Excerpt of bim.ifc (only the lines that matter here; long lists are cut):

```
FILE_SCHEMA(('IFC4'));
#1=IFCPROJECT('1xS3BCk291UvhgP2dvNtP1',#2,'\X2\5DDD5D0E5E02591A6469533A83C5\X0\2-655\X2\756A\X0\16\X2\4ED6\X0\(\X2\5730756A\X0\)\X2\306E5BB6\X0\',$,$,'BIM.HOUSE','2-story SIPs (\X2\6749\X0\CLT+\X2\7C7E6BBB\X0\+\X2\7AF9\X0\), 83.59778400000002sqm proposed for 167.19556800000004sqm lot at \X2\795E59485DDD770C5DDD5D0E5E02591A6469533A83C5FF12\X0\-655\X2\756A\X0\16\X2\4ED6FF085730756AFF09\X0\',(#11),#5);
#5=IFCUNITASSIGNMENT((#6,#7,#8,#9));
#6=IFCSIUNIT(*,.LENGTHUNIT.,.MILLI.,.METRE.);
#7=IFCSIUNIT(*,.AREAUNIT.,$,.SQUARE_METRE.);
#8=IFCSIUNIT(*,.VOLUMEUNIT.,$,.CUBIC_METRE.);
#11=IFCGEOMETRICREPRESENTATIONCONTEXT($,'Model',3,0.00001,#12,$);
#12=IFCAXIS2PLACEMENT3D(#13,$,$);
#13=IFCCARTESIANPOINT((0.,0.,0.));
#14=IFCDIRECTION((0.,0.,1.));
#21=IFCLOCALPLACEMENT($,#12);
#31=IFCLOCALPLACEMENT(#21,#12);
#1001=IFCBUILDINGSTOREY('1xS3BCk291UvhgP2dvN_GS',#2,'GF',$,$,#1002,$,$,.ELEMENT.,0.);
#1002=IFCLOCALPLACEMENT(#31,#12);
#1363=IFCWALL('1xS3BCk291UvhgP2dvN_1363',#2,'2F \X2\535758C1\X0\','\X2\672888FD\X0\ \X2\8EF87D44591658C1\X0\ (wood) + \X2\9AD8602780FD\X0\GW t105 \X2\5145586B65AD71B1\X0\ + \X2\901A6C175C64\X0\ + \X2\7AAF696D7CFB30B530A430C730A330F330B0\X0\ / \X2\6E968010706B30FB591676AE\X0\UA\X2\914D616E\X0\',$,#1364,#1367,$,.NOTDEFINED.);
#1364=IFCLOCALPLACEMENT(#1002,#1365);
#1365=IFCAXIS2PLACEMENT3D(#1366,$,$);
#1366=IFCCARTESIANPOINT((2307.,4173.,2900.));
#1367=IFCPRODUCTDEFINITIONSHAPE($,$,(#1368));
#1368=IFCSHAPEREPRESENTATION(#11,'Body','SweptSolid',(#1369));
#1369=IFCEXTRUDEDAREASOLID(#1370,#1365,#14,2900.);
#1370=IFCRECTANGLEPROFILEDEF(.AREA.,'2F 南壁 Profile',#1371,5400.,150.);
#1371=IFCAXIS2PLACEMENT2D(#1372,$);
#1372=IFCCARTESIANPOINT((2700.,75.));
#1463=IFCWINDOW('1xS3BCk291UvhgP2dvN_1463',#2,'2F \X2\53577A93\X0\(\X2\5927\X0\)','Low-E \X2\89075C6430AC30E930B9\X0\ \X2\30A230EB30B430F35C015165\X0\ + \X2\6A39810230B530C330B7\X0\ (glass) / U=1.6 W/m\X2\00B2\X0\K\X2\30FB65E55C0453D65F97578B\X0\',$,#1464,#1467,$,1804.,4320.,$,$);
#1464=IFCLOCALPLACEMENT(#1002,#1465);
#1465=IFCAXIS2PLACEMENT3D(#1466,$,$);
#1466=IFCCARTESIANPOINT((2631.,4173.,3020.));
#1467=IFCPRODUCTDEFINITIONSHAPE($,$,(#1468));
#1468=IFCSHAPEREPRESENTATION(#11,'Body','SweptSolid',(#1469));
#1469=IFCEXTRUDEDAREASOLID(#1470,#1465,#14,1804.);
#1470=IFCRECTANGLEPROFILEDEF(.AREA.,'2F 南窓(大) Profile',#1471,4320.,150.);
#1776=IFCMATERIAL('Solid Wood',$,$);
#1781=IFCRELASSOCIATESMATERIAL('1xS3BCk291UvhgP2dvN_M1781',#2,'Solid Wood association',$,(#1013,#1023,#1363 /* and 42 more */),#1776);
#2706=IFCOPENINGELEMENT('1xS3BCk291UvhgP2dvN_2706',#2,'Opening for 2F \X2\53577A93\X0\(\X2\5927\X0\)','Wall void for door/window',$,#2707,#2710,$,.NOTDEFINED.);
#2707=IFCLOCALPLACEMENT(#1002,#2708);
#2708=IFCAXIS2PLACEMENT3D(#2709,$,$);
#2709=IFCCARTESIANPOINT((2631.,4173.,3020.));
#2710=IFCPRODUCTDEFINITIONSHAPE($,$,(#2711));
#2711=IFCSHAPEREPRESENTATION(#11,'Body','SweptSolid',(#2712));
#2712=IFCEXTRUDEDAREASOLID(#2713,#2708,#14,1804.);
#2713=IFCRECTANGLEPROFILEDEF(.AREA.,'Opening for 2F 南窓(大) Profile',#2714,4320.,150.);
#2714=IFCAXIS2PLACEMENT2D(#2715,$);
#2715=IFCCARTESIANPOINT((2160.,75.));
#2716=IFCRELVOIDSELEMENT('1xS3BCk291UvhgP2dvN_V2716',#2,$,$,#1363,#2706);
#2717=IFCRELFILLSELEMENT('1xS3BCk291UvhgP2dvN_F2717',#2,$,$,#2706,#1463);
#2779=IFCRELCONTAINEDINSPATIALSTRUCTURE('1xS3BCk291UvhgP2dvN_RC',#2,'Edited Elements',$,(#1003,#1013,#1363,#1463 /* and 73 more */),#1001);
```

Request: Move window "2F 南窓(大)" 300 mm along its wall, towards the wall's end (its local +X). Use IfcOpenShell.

```python
import ifcopenshell
import ifcopenshell.api.geometry
import ifcopenshell.util.placement
import ifcopenshell.util.unit

model = ifcopenshell.open("bim.ifc")
unit_scale = ifcopenshell.util.unit.calculate_unit_scale(model)

window = model.by_guid("1xS3BCk291UvhgP2dvN_1463")
opening = window.FillsVoids[0].RelatingOpeningElement
wall = opening.VoidsElements[0].RelatingBuildingElement

wall_matrix = ifcopenshell.util.placement.get_local_placement(wall.ObjectPlacement)
shift = wall_matrix[:3, 0] * 0.3 / unit_scale
before = ifcopenshell.util.placement.get_local_placement(window.ObjectPlacement)[:3, 3].copy()

# The window is not placed relative to its opening, so move both.
for product in (opening, window):
    matrix = ifcopenshell.util.placement.get_local_placement(product.ObjectPlacement)
    matrix[:3, 3] += shift
    ifcopenshell.api.geometry.edit_object_placement(model, product=product, matrix=matrix, is_si=False)

after = ifcopenshell.util.placement.get_local_placement(window.ObjectPlacement)[:3, 3]
print("window moved by", (after - before).round(3) + 0.0)

model.write("bim_edited.ifc")
```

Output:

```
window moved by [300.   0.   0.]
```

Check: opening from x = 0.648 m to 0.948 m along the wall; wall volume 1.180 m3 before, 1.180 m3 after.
